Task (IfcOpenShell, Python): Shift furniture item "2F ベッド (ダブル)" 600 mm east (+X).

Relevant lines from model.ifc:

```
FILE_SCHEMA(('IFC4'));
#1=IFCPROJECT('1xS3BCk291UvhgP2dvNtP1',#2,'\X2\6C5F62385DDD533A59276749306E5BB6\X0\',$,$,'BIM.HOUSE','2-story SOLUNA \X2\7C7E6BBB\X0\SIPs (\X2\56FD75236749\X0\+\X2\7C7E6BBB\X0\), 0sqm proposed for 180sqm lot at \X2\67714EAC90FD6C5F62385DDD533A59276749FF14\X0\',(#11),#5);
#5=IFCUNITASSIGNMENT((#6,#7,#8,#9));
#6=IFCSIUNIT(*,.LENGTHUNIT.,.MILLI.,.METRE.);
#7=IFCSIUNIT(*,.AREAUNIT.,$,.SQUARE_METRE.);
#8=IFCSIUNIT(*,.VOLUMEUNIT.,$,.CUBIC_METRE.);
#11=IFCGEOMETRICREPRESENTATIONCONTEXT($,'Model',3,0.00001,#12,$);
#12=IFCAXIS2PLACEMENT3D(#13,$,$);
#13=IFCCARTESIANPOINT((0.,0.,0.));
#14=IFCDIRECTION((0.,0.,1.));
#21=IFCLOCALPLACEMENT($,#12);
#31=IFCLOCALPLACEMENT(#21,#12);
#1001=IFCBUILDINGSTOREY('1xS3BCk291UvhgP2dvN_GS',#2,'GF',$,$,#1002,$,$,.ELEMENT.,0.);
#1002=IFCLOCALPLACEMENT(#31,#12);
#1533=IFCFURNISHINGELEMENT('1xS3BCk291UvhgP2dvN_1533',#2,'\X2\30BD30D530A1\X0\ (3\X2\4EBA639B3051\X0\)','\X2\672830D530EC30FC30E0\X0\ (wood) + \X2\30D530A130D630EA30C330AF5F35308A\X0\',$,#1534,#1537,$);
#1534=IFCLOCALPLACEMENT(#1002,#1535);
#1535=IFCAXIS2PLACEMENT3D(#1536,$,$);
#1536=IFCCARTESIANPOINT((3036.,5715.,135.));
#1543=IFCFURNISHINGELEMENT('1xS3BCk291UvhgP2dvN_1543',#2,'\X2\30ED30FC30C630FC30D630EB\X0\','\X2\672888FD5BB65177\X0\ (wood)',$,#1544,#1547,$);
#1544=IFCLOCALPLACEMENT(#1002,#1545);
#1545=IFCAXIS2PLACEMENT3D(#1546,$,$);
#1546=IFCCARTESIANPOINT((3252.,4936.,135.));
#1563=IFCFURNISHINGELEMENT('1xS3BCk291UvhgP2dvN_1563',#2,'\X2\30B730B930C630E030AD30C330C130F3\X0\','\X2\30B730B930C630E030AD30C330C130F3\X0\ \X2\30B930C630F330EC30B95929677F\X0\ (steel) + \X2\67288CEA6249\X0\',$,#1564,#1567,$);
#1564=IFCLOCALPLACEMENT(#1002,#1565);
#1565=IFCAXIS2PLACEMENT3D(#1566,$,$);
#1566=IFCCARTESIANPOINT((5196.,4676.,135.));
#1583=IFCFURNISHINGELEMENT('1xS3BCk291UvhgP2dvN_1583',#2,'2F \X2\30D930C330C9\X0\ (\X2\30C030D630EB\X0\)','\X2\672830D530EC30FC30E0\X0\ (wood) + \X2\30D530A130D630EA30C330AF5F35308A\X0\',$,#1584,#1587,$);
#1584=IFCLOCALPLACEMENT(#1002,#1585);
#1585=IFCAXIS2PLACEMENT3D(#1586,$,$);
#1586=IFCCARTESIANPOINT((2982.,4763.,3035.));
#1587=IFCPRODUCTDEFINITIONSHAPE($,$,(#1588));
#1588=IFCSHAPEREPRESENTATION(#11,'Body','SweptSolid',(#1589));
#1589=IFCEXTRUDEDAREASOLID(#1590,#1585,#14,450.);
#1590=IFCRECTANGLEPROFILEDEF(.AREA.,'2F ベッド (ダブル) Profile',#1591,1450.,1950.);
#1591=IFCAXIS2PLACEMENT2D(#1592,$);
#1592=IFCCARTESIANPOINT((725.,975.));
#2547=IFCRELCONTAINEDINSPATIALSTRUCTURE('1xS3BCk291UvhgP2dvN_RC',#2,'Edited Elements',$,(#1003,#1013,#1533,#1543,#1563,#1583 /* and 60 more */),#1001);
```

```python
import ifcopenshell
import ifcopenshell.api.geometry
import ifcopenshell.util.placement
import ifcopenshell.util.unit

model = ifcopenshell.open("model.ifc")
unit_scale = ifcopenshell.util.unit.calculate_unit_scale(model)

item = model.by_guid("1xS3BCk291UvhgP2dvN_1583")
matrix = ifcopenshell.util.placement.get_local_placement(item.ObjectPlacement)
matrix[0, 3] += 0.6 / unit_scale
ifcopenshell.api.geometry.edit_object_placement(model, product=item, matrix=matrix, is_si=False)

print(ifcopenshell.util.placement.get_local_placement(item.ObjectPlacement).round(3) + 0.0)

model.write("model-out.ifc")
```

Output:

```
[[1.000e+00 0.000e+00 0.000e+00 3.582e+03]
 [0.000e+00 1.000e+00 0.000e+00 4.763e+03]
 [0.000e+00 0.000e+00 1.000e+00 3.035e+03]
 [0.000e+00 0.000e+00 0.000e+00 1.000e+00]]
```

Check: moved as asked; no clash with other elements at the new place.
